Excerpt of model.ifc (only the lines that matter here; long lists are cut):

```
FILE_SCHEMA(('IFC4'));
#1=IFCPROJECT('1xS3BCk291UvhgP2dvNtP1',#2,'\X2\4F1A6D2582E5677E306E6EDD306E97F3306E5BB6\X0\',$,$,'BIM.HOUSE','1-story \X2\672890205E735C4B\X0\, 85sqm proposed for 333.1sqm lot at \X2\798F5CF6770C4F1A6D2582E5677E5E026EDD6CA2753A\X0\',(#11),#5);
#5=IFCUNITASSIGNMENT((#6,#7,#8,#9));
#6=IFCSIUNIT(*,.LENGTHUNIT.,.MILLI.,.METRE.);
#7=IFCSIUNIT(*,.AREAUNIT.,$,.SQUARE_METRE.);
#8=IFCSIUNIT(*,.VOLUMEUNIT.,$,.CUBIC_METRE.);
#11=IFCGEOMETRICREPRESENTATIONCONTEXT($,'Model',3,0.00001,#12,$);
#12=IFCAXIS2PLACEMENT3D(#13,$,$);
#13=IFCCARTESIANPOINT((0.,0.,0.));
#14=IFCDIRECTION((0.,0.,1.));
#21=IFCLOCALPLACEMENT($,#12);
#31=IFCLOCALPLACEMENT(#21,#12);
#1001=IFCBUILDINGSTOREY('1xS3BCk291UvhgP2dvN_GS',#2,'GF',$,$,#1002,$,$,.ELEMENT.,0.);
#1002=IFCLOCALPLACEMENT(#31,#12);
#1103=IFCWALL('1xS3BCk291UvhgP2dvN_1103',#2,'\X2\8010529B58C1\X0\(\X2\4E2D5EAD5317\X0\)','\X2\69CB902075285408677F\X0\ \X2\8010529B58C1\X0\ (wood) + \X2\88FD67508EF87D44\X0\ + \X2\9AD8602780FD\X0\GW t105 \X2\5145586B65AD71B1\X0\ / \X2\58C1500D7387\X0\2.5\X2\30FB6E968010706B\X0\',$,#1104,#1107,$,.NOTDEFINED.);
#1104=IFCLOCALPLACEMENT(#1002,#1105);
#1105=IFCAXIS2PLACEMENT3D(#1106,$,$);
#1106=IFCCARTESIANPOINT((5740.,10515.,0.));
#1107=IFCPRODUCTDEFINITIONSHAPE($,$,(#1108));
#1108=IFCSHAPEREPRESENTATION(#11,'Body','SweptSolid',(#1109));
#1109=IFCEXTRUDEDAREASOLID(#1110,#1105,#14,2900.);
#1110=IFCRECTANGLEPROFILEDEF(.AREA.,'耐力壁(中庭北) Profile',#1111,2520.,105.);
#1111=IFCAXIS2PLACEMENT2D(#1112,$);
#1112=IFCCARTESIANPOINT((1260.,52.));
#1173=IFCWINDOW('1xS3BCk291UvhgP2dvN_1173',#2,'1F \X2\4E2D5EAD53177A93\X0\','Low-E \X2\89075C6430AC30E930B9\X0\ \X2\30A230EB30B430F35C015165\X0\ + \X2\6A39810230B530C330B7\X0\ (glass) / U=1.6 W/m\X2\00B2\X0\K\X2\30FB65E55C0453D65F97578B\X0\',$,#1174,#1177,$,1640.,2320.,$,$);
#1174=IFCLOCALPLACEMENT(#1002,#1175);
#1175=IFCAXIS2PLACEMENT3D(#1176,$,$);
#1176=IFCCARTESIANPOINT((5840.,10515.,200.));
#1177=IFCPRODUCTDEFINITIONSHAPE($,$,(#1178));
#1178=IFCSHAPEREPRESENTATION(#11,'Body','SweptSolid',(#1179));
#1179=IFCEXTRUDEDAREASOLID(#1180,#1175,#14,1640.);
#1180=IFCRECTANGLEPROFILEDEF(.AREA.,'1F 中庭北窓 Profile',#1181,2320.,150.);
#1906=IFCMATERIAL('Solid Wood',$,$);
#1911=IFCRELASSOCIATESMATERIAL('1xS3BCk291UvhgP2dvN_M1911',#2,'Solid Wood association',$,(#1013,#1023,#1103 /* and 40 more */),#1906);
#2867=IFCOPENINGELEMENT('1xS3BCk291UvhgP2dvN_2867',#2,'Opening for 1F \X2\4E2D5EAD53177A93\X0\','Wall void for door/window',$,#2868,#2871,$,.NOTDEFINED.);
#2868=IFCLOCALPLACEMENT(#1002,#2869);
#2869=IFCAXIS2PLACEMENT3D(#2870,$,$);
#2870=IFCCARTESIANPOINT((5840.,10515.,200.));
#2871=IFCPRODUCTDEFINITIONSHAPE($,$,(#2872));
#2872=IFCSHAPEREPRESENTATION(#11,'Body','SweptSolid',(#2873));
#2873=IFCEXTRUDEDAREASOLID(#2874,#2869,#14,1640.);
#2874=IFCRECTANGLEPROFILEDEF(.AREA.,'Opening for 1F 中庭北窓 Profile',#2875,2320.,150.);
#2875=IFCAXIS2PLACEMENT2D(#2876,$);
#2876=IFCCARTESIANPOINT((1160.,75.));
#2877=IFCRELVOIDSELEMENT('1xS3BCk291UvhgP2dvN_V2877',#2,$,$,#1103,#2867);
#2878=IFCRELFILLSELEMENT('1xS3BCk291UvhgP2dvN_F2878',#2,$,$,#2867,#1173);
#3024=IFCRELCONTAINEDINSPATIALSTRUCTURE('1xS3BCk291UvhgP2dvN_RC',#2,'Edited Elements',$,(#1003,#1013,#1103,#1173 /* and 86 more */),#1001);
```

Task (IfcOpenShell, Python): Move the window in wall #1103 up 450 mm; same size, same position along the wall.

```python
import numpy as np
import ifcopenshell
import ifcopenshell.api.geometry
import ifcopenshell.util.placement
import ifcopenshell.util.unit

model = ifcopenshell.open("model.ifc")
unit_scale = ifcopenshell.util.unit.calculate_unit_scale(model)

window = model.by_guid("1xS3BCk291UvhgP2dvN_1173")
opening = window.FillsVoids[0].RelatingOpeningElement
dz = 0.45 / unit_scale

shift = np.array([0.0, 0.0, dz])
# The window is not placed relative to its opening, so move both.
for product in (opening, window):
    matrix = ifcopenshell.util.placement.get_local_placement(product.ObjectPlacement)
    matrix[:3, 3] += shift
    ifcopenshell.api.geometry.edit_object_placement(model, product=product, matrix=matrix, is_si=False)

print(f"moved by {dz * unit_scale:+.3f} m")

model.write("model_edited.ifc")
```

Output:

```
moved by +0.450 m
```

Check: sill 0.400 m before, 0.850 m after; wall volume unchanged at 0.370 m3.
